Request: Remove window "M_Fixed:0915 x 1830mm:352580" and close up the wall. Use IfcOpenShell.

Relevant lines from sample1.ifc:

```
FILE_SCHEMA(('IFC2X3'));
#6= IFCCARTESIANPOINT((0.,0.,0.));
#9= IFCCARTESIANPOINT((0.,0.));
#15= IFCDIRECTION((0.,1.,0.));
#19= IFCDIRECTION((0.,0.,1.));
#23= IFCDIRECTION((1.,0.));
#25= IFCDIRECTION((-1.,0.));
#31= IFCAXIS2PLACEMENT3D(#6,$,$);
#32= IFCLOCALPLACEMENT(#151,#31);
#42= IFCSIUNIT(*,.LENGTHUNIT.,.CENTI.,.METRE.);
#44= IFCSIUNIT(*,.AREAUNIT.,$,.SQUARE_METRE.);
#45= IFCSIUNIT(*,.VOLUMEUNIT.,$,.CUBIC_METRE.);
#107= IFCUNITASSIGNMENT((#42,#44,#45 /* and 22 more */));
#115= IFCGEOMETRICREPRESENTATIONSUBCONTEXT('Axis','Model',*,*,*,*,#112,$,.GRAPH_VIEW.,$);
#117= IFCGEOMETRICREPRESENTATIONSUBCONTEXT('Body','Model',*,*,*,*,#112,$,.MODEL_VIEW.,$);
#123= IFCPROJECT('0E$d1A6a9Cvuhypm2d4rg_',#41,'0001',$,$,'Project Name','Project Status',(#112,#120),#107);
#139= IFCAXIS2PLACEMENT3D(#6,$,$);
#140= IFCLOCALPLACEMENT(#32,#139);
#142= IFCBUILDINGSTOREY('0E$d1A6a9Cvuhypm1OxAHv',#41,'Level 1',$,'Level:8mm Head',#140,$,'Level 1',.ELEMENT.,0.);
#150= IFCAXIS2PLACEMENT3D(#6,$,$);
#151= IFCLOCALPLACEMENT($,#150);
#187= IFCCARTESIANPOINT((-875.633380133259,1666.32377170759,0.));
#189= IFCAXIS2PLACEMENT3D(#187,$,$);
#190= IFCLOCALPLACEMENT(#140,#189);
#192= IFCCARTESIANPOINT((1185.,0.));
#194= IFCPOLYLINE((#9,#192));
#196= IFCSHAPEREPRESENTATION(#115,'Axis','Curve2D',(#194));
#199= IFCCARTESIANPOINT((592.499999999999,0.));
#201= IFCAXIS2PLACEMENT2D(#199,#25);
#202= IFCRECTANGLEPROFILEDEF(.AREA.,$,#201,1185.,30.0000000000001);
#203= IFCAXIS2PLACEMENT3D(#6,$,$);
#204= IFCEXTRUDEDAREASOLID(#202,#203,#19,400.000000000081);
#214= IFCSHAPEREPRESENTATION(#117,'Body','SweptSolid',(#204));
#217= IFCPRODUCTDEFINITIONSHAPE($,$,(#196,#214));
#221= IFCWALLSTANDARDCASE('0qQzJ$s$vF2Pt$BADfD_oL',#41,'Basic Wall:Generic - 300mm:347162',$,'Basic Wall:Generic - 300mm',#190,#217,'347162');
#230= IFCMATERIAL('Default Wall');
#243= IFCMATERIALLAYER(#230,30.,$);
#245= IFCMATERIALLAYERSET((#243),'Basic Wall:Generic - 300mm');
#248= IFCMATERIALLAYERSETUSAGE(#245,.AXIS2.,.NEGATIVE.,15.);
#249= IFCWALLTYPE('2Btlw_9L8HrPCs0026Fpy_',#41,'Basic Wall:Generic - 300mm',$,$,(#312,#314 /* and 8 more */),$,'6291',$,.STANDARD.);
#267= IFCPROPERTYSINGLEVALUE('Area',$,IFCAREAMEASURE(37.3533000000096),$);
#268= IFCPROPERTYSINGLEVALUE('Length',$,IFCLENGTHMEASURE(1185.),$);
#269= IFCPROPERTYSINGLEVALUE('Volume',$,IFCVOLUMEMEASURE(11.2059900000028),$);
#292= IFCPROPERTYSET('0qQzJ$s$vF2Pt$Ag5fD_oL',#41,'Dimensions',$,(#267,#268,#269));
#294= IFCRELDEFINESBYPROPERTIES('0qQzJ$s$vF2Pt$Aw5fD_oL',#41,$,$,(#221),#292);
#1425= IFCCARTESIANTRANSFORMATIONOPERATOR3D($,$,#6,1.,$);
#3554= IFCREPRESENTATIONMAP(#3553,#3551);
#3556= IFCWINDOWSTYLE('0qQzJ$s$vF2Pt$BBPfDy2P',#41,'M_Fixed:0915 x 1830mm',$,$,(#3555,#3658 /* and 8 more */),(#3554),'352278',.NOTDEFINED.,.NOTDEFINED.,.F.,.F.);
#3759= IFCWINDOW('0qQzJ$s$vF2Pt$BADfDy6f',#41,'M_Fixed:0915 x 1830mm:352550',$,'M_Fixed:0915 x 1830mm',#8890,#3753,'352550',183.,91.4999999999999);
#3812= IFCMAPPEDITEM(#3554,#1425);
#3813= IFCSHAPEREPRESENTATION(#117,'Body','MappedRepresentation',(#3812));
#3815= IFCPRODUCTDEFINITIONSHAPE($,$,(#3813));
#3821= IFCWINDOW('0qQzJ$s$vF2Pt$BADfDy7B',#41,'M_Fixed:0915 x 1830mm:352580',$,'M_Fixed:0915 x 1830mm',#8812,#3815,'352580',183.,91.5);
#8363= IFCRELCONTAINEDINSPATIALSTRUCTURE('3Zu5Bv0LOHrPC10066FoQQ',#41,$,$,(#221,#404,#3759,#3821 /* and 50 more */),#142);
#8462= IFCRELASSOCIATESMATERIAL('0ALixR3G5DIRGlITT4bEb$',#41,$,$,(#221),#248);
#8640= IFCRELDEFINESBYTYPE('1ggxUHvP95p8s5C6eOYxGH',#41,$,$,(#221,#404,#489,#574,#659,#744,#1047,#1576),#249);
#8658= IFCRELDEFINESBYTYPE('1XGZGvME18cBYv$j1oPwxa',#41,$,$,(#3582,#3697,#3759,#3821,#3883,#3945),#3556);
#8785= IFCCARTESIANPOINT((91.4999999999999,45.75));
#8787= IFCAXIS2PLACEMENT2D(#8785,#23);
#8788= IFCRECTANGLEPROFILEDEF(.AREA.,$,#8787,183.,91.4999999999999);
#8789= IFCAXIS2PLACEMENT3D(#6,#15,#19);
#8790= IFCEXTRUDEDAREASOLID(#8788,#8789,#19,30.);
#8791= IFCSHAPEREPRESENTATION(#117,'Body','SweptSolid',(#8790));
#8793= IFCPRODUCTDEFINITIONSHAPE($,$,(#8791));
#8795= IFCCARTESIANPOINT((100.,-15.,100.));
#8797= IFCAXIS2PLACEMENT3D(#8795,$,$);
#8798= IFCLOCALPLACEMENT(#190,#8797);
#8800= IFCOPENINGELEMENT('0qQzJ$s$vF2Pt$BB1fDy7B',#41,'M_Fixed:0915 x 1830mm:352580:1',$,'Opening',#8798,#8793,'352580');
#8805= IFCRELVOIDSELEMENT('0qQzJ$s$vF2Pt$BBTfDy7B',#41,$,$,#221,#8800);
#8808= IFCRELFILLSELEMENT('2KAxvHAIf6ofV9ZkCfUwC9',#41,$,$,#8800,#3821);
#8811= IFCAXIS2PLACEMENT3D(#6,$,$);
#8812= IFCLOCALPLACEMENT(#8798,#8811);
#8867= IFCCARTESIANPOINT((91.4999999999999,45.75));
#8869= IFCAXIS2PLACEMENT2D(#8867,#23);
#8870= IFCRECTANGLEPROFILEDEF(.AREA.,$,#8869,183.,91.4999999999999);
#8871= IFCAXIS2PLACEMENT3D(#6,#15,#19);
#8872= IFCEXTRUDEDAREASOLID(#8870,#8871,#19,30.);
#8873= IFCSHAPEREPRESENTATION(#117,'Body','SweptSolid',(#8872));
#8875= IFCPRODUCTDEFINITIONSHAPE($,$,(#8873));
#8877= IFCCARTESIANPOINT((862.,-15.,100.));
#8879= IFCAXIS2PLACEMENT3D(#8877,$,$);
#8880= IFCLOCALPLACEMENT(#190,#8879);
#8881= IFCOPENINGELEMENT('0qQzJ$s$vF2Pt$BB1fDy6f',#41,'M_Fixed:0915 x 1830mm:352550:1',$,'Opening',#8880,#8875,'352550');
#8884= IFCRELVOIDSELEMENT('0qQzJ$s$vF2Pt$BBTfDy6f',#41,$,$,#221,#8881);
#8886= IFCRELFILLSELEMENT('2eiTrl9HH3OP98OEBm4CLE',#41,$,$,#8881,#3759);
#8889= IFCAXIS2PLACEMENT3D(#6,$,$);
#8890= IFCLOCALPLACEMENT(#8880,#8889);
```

```python
import ifcopenshell
import ifcopenshell.api.feature
import ifcopenshell.api.pset
import ifcopenshell.api.root
import ifcopenshell.geom
import ifcopenshell.util.element
import ifcopenshell.util.shape
import ifcopenshell.util.unit

model = ifcopenshell.open("sample1.ifc")
area_scale = ifcopenshell.util.unit.calculate_unit_scale(model, "AREAUNIT")
volume_scale = ifcopenshell.util.unit.calculate_unit_scale(model, "VOLUMEUNIT")
settings = ifcopenshell.geom.settings()


def volume(element):
    """Net volume in cubic metres, openings subtracted."""
    shape = ifcopenshell.geom.create_shape(settings, element)
    return ifcopenshell.util.shape.get_volume(shape.geometry)


window = model.by_guid("0qQzJ$s$vF2Pt$BADfDy7B")
opening = window.FillsVoids[0].RelatingOpeningElement
wall = opening.VoidsElements[0].RelatingBuildingElement
before = volume(wall)

ifcopenshell.api.root.remove_product(model, product=window)
ifcopenshell.api.feature.remove_feature(model, feature=opening)

after = volume(wall)
thickness = 0.3  # wall thickness in metres

# Update the wall's stored quantities.
pset = model.by_id(ifcopenshell.util.element.get_pset(wall, "Dimensions", should_inherit=False)["id"])
ifcopenshell.api.pset.edit_pset(model, pset=pset, properties={
    "Area": model.create_entity("IfcAreaMeasure", after / thickness / area_scale),
    "Volume": model.create_entity("IfcVolumeMeasure", after / volume_scale),
})

print(f"wall volume {before:.3f} -> {after:.3f} m3")

model.write("sample1_updated.ifc")
```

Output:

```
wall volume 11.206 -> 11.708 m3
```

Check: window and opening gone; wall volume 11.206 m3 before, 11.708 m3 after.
